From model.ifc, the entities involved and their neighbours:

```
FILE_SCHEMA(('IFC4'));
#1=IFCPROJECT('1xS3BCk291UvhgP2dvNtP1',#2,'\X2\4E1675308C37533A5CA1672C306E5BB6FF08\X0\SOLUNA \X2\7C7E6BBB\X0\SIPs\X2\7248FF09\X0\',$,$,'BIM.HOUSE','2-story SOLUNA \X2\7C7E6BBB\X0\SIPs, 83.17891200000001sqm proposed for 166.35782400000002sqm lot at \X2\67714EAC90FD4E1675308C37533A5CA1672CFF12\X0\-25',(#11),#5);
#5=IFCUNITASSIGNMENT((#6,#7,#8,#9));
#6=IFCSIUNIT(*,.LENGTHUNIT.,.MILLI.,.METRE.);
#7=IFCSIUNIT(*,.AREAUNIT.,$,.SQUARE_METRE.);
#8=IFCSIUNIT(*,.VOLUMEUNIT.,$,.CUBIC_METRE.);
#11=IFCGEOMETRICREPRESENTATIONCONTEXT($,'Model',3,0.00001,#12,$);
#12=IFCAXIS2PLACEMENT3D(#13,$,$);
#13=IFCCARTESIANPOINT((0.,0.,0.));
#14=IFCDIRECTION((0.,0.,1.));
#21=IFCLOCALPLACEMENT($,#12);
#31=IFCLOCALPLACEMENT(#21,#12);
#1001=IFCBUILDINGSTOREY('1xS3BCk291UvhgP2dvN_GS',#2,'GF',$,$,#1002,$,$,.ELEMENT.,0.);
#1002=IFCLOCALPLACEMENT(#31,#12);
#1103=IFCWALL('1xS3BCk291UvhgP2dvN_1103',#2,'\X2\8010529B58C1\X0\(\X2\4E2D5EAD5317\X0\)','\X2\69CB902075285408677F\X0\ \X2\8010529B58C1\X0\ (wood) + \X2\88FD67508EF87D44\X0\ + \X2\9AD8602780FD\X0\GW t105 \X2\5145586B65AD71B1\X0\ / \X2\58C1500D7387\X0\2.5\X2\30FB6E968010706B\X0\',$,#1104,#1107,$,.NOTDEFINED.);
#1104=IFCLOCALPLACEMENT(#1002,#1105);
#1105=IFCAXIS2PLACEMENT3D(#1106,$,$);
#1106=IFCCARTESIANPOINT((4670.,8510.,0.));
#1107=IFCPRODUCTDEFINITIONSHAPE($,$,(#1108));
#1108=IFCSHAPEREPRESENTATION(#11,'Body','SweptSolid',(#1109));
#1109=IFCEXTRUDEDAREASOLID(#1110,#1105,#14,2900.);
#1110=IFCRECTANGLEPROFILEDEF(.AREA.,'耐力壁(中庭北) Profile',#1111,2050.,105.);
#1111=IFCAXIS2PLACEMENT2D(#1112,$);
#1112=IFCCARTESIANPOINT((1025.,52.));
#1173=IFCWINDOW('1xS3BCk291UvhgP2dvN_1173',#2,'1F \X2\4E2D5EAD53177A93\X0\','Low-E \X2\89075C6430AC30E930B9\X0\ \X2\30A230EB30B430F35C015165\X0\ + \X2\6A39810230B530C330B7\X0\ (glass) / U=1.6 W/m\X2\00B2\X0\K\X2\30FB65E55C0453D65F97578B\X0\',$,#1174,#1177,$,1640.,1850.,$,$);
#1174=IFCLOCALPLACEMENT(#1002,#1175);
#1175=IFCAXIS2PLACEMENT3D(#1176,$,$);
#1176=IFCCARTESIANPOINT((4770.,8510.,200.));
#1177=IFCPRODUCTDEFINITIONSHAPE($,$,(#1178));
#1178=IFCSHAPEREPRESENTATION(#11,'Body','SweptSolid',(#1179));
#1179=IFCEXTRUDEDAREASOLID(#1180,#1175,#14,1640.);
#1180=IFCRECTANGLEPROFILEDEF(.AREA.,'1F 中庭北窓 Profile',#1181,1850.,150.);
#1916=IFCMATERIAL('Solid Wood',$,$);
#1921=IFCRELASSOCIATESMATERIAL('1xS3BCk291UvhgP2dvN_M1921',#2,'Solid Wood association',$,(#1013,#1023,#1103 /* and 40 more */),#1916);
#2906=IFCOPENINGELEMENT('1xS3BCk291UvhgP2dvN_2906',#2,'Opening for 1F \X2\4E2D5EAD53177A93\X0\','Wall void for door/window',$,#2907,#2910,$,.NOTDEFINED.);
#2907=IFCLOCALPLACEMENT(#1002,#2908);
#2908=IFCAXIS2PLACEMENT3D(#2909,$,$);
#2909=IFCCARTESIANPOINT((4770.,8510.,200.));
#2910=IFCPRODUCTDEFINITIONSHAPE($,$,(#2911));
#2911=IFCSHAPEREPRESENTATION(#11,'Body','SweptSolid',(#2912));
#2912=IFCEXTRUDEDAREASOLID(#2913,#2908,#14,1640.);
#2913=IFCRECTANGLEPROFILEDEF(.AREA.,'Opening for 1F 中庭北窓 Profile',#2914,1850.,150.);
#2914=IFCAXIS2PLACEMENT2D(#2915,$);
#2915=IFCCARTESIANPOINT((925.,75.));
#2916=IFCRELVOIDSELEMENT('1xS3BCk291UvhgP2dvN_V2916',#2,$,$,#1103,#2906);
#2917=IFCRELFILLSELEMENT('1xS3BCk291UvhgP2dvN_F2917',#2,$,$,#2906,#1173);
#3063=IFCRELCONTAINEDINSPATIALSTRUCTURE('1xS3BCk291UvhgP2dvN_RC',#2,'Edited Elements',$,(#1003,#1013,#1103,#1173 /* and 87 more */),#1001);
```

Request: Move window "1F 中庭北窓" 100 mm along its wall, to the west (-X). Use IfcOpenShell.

```python
import ifcopenshell
import ifcopenshell.api.geometry
import ifcopenshell.util.placement
import ifcopenshell.util.unit

model = ifcopenshell.open("model.ifc")
unit_scale = ifcopenshell.util.unit.calculate_unit_scale(model)

window = model.by_id(1173)
opening = window.FillsVoids[0].RelatingOpeningElement
wall = opening.VoidsElements[0].RelatingBuildingElement

wall_matrix = ifcopenshell.util.placement.get_local_placement(wall.ObjectPlacement)
shift = wall_matrix[:3, 0] * -0.1 / unit_scale
before = ifcopenshell.util.placement.get_local_placement(window.ObjectPlacement)[:3, 3].copy()

# The window is not placed relative to its opening, so move both.
for product in (opening, window):
    matrix = ifcopenshell.util.placement.get_local_placement(product.ObjectPlacement)
    matrix[:3, 3] += shift
    ifcopenshell.api.geometry.edit_object_placement(model, product=product, matrix=matrix, is_si=False)

after = ifcopenshell.util.placement.get_local_placement(window.ObjectPlacement)[:3, 3]
print("window moved by", (after - before).round(3) + 0.0)

model.write("model-out.ifc")
```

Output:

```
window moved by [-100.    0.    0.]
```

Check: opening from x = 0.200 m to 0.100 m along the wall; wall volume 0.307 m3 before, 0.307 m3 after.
